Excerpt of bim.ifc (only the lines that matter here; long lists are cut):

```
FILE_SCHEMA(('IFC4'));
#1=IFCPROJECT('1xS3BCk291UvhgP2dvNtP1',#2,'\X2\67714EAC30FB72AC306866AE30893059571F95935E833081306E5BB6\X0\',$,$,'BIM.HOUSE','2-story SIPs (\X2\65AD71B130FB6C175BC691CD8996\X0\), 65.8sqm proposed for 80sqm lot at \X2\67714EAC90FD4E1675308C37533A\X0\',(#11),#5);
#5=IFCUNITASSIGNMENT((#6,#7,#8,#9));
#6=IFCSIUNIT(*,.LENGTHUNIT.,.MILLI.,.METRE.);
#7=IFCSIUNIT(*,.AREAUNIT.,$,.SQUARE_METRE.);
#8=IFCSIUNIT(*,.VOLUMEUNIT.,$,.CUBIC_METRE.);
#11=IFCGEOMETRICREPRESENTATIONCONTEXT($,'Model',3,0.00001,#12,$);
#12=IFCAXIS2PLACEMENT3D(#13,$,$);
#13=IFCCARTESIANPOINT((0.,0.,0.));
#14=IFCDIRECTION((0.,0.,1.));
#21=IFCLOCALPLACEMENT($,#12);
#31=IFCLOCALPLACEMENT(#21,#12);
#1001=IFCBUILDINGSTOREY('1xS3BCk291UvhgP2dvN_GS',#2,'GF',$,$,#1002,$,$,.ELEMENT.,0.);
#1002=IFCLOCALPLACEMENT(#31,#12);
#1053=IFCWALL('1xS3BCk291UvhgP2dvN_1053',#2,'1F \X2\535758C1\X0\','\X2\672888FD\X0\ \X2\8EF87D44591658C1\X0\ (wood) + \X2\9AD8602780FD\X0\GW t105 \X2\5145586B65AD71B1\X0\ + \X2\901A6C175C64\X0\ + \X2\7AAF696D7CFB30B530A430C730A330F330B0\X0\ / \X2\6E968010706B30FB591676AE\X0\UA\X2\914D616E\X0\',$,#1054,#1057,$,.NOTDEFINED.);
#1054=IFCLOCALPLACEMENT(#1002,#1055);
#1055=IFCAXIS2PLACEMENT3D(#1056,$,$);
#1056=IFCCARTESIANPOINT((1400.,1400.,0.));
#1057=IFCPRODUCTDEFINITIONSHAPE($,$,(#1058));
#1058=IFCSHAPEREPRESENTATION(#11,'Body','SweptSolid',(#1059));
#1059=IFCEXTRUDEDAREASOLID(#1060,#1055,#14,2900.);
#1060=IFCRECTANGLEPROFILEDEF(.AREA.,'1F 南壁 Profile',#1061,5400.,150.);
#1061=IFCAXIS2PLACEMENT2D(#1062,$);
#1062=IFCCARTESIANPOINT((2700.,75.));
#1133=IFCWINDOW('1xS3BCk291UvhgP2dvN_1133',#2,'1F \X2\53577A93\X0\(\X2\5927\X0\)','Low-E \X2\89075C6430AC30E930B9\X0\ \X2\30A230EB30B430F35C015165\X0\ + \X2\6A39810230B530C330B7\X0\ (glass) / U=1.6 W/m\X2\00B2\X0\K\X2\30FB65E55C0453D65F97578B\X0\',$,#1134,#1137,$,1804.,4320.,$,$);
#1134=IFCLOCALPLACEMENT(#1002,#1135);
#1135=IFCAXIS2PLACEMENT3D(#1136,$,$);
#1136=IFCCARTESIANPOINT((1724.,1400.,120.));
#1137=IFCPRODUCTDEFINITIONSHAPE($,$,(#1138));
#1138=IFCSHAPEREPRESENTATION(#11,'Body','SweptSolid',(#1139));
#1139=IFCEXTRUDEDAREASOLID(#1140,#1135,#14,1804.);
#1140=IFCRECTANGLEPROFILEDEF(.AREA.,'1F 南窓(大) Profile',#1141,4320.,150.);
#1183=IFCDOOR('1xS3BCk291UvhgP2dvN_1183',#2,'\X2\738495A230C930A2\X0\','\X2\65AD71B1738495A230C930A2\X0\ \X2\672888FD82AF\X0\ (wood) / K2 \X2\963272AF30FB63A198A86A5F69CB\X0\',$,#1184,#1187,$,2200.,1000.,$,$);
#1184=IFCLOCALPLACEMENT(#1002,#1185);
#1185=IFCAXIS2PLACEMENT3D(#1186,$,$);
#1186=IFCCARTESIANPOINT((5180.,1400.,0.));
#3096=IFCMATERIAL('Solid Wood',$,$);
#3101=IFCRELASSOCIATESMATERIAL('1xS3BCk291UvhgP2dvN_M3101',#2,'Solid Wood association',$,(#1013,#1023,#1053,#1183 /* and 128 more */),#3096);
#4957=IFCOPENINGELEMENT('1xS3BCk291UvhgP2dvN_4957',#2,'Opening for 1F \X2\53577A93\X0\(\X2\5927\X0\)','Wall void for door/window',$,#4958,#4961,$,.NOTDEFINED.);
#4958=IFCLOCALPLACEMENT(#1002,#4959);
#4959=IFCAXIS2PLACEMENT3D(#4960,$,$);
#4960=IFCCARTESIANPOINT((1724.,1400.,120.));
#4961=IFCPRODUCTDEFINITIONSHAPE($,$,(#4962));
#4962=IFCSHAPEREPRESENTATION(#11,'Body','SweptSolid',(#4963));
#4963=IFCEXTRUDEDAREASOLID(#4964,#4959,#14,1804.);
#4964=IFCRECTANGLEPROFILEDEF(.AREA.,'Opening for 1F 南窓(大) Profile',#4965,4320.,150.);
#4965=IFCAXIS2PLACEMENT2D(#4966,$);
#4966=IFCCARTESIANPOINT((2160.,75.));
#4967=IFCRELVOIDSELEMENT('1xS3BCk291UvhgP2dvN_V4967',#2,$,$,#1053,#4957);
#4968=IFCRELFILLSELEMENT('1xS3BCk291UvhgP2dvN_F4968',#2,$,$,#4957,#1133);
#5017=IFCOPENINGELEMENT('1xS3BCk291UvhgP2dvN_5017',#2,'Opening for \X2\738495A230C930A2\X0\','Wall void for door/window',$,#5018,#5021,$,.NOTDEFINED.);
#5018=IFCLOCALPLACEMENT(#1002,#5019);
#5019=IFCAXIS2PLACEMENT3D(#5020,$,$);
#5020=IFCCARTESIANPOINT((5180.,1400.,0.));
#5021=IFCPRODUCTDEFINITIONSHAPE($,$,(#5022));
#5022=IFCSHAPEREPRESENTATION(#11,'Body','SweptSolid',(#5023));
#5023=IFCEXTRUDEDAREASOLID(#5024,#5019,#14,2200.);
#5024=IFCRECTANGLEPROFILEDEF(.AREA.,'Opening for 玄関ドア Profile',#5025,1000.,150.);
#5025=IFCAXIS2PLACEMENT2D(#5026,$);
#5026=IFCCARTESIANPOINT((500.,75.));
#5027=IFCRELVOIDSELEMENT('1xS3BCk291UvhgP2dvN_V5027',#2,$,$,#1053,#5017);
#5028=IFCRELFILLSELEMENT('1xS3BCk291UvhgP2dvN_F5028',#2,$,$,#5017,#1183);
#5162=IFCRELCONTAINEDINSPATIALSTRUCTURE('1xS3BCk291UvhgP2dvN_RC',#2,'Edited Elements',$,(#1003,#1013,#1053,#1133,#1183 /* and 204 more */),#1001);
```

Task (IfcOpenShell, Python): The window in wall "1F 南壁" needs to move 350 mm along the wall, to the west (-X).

```python
import ifcopenshell
import ifcopenshell.api.geometry
import ifcopenshell.util.placement

model = ifcopenshell.open("bim.ifc")

window = model.by_id(1133)
opening = window.FillsVoids[0].RelatingOpeningElement
wall = opening.VoidsElements[0].RelatingBuildingElement

wall_matrix = ifcopenshell.util.placement.get_local_placement(wall.ObjectPlacement)
shift = wall_matrix[:3, 0] * -350.0
before = ifcopenshell.util.placement.get_local_placement(window.ObjectPlacement)[:3, 3].copy()

# The window is not placed relative to its opening, so move both.
for product in (opening, window):
    matrix = ifcopenshell.util.placement.get_local_placement(product.ObjectPlacement)
    matrix[:3, 3] += shift
    ifcopenshell.api.geometry.edit_object_placement(model, product=product, matrix=matrix, is_si=False)

after = ifcopenshell.util.placement.get_local_placement(window.ObjectPlacement)[:3, 3]
print("window moved by", (after - before).round(3) + 0.0)

model.write("bim-out.ifc")
```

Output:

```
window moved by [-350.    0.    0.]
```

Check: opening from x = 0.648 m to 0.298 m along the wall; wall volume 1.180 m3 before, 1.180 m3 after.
